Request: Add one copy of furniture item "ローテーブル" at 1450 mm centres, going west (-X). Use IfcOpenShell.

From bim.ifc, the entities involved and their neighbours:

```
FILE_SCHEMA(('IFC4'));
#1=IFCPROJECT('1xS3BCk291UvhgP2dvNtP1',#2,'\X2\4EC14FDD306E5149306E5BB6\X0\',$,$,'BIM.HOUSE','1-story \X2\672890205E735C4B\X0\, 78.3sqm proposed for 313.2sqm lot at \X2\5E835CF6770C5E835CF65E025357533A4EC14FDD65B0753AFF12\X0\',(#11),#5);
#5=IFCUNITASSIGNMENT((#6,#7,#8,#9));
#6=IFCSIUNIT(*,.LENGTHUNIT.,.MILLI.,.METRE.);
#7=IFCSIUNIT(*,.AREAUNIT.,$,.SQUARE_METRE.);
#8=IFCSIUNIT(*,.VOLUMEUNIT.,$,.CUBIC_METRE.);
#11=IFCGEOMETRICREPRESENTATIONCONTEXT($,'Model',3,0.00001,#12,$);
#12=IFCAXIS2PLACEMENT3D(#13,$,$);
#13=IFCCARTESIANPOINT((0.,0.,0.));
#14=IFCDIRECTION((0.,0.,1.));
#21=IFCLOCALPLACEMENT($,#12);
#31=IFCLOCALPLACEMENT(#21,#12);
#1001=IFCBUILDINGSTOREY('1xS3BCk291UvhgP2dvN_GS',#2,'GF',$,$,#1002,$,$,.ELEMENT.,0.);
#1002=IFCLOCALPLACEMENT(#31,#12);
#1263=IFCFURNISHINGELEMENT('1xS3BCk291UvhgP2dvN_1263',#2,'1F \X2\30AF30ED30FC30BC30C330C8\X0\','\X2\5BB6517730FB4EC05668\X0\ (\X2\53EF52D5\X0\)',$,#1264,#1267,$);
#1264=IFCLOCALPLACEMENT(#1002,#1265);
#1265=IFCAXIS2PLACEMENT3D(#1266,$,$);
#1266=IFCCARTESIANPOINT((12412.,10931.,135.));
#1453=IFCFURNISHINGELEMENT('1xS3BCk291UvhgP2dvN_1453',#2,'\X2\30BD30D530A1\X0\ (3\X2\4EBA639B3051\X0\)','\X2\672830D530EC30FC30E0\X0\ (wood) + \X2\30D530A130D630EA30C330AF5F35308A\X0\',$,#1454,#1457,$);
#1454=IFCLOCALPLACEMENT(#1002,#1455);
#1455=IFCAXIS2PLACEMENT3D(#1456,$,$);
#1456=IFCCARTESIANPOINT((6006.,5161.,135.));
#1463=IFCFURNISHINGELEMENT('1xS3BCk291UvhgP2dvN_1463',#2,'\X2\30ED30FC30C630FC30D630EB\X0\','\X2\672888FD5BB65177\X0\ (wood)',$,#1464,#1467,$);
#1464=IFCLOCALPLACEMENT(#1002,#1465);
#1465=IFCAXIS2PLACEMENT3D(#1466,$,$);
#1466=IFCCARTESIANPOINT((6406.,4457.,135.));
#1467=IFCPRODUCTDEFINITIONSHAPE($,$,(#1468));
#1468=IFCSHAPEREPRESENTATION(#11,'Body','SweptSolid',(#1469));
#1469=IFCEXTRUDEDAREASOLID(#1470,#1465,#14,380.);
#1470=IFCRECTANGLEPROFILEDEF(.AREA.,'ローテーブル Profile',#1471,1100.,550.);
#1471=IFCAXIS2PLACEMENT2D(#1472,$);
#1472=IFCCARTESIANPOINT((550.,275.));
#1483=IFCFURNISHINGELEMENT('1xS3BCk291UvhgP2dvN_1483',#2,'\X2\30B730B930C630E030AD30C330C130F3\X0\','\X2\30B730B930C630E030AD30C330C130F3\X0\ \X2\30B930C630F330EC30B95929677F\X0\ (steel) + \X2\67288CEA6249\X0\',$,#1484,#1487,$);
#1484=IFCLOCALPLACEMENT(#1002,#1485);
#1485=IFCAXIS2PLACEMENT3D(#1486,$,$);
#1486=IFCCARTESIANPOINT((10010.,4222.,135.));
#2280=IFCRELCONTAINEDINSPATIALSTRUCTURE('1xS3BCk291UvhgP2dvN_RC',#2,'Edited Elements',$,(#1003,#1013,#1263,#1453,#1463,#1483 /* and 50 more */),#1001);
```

```python
import numpy as np
import ifcopenshell
import ifcopenshell.api.geometry
import ifcopenshell.api.root
import ifcopenshell.util.element
import ifcopenshell.util.placement
import ifcopenshell.util.unit

model = ifcopenshell.open("bim.ifc")
unit_scale = ifcopenshell.util.unit.calculate_unit_scale(model)


def reuse_history(source, copy):
    """copy_class also copies each property set's owner history, people and application; keep the originals."""
    for rel in copy.IsDefinedBy:
        if rel.is_a("IfcRelDefinesByProperties") and (history := rel.RelatingPropertyDefinition.OwnerHistory):
            rel.RelatingPropertyDefinition.OwnerHistory = source.OwnerHistory
            ifcopenshell.util.element.remove_deep2(model, history)


source = model.by_guid("1xS3BCk291UvhgP2dvN_1463")
base = ifcopenshell.util.placement.get_local_placement(source.ObjectPlacement)
step = np.array([-1.0, 0.0, 0.0]) * 1.45 / unit_scale

for i in range(1, 2):
    copy = ifcopenshell.api.root.copy_class(model, product=source)
    copy.Representation = ifcopenshell.util.element.copy_deep(
        model, source.Representation, exclude=["IfcGeometricRepresentationContext", "IfcRepresentationMap"]
    )
    reuse_history(source, copy)
    matrix = base.copy()
    matrix[:3, 3] += i * step
    print("added at", matrix[:3, 3].round(3) + 0.0)
    ifcopenshell.api.geometry.edit_object_placement(model, product=copy, matrix=matrix, is_si=False)

model.write("bim_rev.ifc")
```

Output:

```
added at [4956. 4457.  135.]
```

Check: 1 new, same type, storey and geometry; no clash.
